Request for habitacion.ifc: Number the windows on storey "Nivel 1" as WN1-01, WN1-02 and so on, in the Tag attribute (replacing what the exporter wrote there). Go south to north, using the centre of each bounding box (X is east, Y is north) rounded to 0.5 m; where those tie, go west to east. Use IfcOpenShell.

First a look at what the model holds.

```python
import ifcopenshell
import ifcopenshell.util.element
import ifcopenshell.util.placement

model = ifcopenshell.open("habitacion.ifc")
print(model.schema)
storey = next(s for s in model.by_type("IfcBuildingStorey") if s.Name == "Nivel 1")
windows = [e for e in ifcopenshell.util.element.get_decomposition(storey) if e.is_a("IfcWindow")]
for e in sorted(windows, key=lambda e: e.id()):
    origin = ifcopenshell.util.placement.get_local_placement(e.ObjectPlacement)[:3, 3]
    print(e.id(), e.Tag, e.Name, origin.round(2) + 0.0, sep=" | ")
```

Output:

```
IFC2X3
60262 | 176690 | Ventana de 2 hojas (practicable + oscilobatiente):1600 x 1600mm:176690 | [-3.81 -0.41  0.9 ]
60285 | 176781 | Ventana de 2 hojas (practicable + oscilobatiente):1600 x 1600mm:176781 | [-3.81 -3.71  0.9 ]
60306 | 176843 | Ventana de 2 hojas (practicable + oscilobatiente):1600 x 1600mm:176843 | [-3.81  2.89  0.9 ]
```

```python
import ifcopenshell
import ifcopenshell.geom
import ifcopenshell.util.element
import ifcopenshell.util.shape

model = ifcopenshell.open("habitacion.ifc")
settings = ifcopenshell.geom.settings()
settings.set("use-world-coords", True)


def centre(element):
    shape = ifcopenshell.geom.create_shape(settings, element)
    return ifcopenshell.util.shape.get_bbox_centroid(shape.geometry)


storey = next(s for s in model.by_type("IfcBuildingStorey") if s.Name == "Nivel 1")
windows = [e for e in ifcopenshell.util.element.get_decomposition(storey) if e.is_a("IfcWindow")]

# Insertion points can sit at a corner or the storey origin, so sort by the geometry (in metres).
centres = {e: centre(e) for e in windows}
windows.sort(key=lambda e: (round(centres[e][1] / 0.5), centres[e][0]))

for i, e in enumerate(windows, start=1):
    number = f"WN1-{i:02d}"
    e.Tag = number
    print(e.id(), number)

model.write("habitacion_updated.ifc")
```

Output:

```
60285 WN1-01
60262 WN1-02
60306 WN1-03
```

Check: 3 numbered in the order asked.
